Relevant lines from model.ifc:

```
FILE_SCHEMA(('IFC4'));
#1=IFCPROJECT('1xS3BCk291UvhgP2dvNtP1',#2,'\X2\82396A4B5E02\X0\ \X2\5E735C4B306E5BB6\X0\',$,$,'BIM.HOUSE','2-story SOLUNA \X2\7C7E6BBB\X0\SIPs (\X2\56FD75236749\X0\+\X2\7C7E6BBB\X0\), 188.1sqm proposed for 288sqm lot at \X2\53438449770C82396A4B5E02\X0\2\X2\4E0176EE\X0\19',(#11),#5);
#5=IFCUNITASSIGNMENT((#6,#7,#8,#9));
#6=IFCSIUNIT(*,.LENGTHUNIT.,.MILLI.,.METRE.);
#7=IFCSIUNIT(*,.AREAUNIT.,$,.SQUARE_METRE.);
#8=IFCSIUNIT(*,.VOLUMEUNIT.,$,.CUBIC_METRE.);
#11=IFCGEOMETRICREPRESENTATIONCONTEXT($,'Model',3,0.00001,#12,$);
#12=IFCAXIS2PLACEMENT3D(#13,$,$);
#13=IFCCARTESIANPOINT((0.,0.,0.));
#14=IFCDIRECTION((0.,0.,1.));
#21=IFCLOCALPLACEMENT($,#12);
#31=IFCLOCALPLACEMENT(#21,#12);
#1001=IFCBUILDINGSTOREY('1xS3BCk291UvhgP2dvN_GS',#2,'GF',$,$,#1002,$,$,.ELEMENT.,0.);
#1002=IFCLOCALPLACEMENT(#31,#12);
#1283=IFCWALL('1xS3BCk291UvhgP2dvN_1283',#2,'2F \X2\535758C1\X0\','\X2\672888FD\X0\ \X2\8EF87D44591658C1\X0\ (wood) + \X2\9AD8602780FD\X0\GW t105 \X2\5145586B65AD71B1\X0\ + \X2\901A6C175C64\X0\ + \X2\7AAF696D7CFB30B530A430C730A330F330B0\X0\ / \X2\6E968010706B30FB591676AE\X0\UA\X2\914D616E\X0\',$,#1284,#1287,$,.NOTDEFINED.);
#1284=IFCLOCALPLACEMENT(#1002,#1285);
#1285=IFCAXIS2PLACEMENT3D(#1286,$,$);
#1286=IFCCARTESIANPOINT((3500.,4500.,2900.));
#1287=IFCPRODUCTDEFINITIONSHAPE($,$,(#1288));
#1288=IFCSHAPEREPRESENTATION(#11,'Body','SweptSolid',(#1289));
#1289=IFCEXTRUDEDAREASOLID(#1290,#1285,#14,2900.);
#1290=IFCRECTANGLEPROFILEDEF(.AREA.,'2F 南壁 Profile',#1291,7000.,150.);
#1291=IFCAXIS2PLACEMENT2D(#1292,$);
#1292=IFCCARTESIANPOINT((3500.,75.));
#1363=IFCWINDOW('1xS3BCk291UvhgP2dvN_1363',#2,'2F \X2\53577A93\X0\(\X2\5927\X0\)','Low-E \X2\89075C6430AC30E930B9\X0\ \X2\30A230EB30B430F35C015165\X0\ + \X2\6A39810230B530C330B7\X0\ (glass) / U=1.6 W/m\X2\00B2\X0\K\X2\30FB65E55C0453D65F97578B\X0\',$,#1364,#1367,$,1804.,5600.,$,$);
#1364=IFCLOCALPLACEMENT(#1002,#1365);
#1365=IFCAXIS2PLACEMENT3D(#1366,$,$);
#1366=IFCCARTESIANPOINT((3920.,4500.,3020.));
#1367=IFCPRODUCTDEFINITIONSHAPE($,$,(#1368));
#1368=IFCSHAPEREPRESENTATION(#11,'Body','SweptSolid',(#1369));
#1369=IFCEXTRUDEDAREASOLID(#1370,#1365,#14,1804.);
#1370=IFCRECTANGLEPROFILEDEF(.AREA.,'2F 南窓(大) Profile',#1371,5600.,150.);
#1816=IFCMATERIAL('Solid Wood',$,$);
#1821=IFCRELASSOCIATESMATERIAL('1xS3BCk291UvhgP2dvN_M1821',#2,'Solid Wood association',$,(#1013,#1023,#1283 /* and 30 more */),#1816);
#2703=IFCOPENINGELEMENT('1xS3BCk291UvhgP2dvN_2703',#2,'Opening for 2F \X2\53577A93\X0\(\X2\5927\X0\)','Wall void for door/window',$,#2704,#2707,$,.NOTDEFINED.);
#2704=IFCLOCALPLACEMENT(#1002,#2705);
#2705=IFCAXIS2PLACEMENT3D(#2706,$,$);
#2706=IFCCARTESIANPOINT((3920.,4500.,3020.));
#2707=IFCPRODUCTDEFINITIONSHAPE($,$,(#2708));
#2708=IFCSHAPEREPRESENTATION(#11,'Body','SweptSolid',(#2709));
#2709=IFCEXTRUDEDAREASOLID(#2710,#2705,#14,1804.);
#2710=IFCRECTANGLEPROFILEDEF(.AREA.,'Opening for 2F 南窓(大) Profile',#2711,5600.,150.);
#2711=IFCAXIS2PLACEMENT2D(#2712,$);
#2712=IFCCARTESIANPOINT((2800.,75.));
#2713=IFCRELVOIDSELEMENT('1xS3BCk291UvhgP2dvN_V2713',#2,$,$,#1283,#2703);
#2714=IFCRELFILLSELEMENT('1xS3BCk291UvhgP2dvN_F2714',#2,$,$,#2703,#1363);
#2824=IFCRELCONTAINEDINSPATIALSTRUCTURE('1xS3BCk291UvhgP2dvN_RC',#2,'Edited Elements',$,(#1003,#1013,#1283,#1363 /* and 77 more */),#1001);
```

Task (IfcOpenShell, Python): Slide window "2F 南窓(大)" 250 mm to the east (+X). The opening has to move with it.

```python
import ifcopenshell
import ifcopenshell.api.geometry
import ifcopenshell.util.placement
import ifcopenshell.util.unit

model = ifcopenshell.open("model.ifc")
unit_scale = ifcopenshell.util.unit.calculate_unit_scale(model)

window = model.by_guid("1xS3BCk291UvhgP2dvN_1363")
opening = window.FillsVoids[0].RelatingOpeningElement
wall = opening.VoidsElements[0].RelatingBuildingElement

wall_matrix = ifcopenshell.util.placement.get_local_placement(wall.ObjectPlacement)
shift = wall_matrix[:3, 0] * 0.25 / unit_scale
before = ifcopenshell.util.placement.get_local_placement(window.ObjectPlacement)[:3, 3].copy()

# The window is not placed relative to its opening, so move both.
for product in (opening, window):
    matrix = ifcopenshell.util.placement.get_local_placement(product.ObjectPlacement)
    matrix[:3, 3] += shift
    ifcopenshell.api.geometry.edit_object_placement(model, product=product, matrix=matrix, is_si=False)

after = ifcopenshell.util.placement.get_local_placement(window.ObjectPlacement)[:3, 3]
print("window moved by", (after - before).round(3) + 0.0)

model.write("model-out.ifc")
```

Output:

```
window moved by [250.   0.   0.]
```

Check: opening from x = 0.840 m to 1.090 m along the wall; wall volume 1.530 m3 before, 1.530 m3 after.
